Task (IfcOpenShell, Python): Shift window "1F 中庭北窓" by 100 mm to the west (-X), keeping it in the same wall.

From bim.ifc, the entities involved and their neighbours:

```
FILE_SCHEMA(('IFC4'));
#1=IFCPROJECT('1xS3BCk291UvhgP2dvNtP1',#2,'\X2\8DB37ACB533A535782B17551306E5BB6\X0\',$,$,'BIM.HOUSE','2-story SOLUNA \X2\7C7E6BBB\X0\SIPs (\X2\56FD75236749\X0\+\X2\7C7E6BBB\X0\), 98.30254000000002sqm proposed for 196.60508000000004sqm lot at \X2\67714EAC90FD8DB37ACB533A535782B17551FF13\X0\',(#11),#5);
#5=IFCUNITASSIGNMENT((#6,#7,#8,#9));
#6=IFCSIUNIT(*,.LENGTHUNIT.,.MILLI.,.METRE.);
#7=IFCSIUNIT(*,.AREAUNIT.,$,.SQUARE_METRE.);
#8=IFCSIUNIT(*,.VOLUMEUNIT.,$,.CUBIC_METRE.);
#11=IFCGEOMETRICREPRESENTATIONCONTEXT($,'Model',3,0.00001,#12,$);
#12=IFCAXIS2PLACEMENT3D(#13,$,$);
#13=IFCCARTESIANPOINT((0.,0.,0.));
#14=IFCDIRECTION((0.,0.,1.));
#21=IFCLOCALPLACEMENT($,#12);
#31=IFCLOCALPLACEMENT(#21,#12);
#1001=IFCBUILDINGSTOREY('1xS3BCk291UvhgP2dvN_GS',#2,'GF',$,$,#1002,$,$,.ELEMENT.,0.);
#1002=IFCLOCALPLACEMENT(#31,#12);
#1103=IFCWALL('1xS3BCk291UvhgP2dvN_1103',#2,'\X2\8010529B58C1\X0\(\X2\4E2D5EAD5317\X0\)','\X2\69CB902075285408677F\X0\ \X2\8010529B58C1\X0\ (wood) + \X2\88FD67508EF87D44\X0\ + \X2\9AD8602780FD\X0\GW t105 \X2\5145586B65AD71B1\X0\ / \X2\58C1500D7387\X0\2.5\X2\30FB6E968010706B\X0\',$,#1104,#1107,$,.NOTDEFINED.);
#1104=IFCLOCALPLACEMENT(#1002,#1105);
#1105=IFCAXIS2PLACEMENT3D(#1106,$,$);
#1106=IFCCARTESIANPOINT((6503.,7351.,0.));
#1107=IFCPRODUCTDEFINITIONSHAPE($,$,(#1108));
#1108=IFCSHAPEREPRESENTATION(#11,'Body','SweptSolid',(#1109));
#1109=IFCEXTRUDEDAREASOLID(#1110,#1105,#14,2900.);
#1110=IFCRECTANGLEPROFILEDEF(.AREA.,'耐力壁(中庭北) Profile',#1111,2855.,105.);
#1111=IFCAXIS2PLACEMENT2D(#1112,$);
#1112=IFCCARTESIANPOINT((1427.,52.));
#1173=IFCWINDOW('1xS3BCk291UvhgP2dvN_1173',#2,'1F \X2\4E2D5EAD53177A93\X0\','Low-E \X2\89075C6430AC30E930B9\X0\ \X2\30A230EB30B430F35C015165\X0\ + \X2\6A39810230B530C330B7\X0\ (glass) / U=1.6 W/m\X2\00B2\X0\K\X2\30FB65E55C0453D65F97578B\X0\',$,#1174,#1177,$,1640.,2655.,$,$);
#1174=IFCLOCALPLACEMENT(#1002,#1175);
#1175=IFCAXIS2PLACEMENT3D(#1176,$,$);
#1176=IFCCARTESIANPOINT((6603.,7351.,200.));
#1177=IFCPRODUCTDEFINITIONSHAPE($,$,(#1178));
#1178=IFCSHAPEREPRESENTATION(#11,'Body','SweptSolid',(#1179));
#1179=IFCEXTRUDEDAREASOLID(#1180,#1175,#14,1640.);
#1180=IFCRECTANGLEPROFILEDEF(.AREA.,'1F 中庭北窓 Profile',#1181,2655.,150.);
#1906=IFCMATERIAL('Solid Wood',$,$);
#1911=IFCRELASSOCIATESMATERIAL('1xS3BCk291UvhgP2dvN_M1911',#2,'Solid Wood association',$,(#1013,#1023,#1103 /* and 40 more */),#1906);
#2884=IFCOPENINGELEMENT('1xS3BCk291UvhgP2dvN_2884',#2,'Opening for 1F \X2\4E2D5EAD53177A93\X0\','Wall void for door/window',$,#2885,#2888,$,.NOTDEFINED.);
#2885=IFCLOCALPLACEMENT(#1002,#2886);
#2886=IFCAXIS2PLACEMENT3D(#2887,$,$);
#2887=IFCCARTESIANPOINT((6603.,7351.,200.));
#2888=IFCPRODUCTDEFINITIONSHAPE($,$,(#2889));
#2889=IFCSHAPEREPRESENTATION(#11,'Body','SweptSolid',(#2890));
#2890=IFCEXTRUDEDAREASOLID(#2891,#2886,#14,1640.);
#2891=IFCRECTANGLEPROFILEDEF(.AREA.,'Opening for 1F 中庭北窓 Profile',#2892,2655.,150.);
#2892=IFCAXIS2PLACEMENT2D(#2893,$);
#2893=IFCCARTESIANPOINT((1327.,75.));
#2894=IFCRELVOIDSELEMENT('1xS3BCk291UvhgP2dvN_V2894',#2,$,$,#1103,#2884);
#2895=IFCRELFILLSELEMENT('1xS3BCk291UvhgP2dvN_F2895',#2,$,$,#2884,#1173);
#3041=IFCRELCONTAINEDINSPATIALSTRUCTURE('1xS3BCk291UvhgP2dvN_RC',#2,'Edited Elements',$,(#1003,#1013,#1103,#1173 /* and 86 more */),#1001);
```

```python
import ifcopenshell
import ifcopenshell.api.geometry
import ifcopenshell.util.placement

model = ifcopenshell.open("bim.ifc")

window = model.by_guid("1xS3BCk291UvhgP2dvN_1173")
opening = window.FillsVoids[0].RelatingOpeningElement
wall = opening.VoidsElements[0].RelatingBuildingElement

wall_matrix = ifcopenshell.util.placement.get_local_placement(wall.ObjectPlacement)
shift = wall_matrix[:3, 0] * -100.0
before = ifcopenshell.util.placement.get_local_placement(window.ObjectPlacement)[:3, 3].copy()

# The window is not placed relative to its opening, so move both.
for product in (opening, window):
    matrix = ifcopenshell.util.placement.get_local_placement(product.ObjectPlacement)
    matrix[:3, 3] += shift
    ifcopenshell.api.geometry.edit_object_placement(model, product=product, matrix=matrix, is_si=False)

after = ifcopenshell.util.placement.get_local_placement(window.ObjectPlacement)[:3, 3]
print("window moved by", (after - before).round(3) + 0.0)

model.write("bim_updated.ifc")
```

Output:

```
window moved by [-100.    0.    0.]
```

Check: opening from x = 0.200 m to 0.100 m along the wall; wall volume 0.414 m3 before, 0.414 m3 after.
